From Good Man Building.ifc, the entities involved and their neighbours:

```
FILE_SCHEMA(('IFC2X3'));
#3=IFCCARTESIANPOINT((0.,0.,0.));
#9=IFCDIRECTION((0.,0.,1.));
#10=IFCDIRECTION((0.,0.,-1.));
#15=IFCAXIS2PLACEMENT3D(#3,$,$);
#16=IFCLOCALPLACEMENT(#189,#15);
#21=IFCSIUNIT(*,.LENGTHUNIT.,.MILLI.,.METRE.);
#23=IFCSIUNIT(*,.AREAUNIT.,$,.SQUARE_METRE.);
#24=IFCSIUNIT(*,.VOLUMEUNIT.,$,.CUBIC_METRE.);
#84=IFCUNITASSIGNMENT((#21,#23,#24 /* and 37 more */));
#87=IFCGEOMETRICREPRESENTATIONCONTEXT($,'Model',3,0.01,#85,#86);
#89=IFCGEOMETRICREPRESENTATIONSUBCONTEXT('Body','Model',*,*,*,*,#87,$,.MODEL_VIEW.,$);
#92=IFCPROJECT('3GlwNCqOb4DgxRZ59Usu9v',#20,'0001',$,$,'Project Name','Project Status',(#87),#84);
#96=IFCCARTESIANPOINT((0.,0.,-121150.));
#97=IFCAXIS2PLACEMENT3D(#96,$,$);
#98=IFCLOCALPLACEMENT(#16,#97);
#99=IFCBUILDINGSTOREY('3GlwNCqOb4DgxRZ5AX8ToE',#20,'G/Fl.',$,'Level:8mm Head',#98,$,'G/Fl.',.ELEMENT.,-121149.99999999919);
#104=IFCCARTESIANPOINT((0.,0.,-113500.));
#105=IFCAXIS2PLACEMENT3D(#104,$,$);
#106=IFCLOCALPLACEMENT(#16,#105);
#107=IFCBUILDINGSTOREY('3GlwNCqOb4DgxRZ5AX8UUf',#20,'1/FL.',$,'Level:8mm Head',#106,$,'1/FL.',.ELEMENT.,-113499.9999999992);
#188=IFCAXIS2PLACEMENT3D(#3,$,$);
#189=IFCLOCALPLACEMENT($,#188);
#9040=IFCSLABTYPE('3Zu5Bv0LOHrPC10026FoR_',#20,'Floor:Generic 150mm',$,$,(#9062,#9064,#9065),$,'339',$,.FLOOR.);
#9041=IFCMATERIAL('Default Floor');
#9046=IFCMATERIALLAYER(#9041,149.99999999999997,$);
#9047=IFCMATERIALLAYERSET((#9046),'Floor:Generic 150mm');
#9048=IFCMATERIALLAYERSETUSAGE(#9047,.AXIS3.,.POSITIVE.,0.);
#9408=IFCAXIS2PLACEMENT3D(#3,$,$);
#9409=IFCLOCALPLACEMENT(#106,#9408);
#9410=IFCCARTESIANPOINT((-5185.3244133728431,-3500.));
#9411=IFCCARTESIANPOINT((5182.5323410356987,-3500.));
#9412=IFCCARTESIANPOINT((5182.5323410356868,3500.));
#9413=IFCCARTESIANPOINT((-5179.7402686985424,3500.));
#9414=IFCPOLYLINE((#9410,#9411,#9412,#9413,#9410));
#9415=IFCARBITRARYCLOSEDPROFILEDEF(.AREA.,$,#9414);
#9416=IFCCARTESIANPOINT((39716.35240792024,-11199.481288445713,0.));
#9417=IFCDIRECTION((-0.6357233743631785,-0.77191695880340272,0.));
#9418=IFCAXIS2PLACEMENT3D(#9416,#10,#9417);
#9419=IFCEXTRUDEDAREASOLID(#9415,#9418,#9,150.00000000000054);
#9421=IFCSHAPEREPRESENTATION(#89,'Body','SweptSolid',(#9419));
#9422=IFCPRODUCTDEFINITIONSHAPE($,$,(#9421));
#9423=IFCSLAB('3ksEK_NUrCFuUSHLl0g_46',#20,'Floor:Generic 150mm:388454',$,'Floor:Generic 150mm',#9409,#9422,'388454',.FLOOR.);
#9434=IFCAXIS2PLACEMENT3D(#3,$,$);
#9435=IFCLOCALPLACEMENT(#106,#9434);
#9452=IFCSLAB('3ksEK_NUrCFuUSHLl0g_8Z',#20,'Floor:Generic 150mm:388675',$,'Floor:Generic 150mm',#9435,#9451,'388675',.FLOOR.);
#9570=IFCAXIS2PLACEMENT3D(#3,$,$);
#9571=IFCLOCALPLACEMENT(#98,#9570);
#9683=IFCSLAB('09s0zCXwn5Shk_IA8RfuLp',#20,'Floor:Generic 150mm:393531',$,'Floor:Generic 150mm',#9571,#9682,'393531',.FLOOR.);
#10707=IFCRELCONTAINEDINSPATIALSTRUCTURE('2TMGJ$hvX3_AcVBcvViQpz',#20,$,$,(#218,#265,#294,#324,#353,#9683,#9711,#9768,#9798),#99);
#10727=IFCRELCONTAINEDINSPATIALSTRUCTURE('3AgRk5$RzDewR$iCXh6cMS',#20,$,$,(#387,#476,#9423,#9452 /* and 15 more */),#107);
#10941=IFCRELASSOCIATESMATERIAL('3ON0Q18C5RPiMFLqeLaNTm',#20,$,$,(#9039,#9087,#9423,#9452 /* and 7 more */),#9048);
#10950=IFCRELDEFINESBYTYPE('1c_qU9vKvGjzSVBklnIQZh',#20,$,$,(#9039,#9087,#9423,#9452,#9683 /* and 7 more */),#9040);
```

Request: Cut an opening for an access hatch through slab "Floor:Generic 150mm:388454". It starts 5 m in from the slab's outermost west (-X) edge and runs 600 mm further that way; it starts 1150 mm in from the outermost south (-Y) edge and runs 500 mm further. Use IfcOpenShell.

```python
import numpy as np
import ifcopenshell
import ifcopenshell.api.feature
import ifcopenshell.api.geometry
import ifcopenshell.api.root
import ifcopenshell.geom
import ifcopenshell.util.placement
import ifcopenshell.util.representation
import ifcopenshell.util.shape
import ifcopenshell.util.unit

model = ifcopenshell.open("Good Man Building.ifc")
unit_scale = ifcopenshell.util.unit.calculate_unit_scale(model)
settings = ifcopenshell.geom.settings()


def volume(element):
    """Net volume in cubic metres, openings subtracted."""
    shape = ifcopenshell.geom.create_shape(settings, element)
    return ifcopenshell.util.shape.get_volume(shape.geometry)


slab = model.by_guid("3ksEK_NUrCFuUSHLl0g_46")
before = volume(slab)

# Extent in the slab's own axes, in metres. The edges named are its -X and -Y sides.
slab_shape = ifcopenshell.geom.create_shape(settings, slab)
vertices = ifcopenshell.util.shape.get_vertices(slab_shape.geometry)
x_min, y_min, bottom = vertices.min(axis=0)
top = vertices[:, 2].max()

opening = ifcopenshell.api.root.create_entity(model, ifc_class="IfcOpeningElement", name="Access hatch opening")
context = ifcopenshell.util.representation.get_context(model, "Model", "Body", "MODEL_VIEW")
width, depth = 0.6, 0.5
outline = [(0.0, 0.0), (width, 0.0), (width, depth), (0.0, depth), (0.0, 0.0)]
# Overshoot both faces by 50 mm so the cut is clean.
shape = ifcopenshell.api.geometry.add_slab_representation(
    model, context=context, depth=top - bottom + 0.1, polyline=outline
)
ifcopenshell.api.geometry.assign_representation(model, product=opening, representation=shape)

matrix = ifcopenshell.util.placement.get_local_placement(slab.ObjectPlacement)
matrix[:, 3] = matrix @ np.append(np.array([x_min + 5, y_min + 1.15, bottom - 0.05]) / unit_scale, 1.0)
ifcopenshell.api.geometry.edit_object_placement(model, product=opening, matrix=matrix, is_si=False)
ifcopenshell.api.feature.add_feature(model, feature=opening, element=slab)

after = volume(slab)

print(f"slab volume {before:.3f} -> {after:.3f} m3")

model.write("Good Man Building_updated.ifc")
```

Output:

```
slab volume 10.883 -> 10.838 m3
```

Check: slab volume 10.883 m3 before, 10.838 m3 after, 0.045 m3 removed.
